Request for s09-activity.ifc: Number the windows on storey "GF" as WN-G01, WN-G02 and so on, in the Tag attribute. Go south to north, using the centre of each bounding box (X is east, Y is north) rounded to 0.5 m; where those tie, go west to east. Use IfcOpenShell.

First a look at what the model holds.

```python
import ifcopenshell
import ifcopenshell.util.element
import ifcopenshell.util.placement

model = ifcopenshell.open("s09-activity.ifc")
print(model.schema)
storey = next(s for s in model.by_type("IfcBuildingStorey") if s.Name == "GF")
windows = [e for e in ifcopenshell.util.element.get_decomposition(storey) if e.is_a("IfcWindow")]
for e in sorted(windows, key=lambda e: e.id()):
    origin = ifcopenshell.util.placement.get_local_placement(e.ObjectPlacement)[:3, 3]
    print(e.id(), e.Tag, e.Name, origin.round(2) + 0.0, sep=" | ")
```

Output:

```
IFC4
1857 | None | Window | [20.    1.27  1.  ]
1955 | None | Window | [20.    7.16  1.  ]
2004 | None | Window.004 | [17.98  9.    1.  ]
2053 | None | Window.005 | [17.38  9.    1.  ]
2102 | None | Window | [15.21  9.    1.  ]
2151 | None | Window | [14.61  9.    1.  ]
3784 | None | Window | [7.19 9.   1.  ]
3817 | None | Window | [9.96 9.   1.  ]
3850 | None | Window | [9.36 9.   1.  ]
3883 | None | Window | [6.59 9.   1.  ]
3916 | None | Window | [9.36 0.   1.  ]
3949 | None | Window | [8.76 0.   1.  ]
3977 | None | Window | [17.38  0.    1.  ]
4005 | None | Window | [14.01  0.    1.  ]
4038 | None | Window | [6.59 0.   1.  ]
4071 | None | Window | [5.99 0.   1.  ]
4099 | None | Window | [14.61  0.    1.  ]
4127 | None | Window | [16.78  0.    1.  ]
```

```python
import ifcopenshell
import ifcopenshell.geom
import ifcopenshell.util.element
import ifcopenshell.util.shape

model = ifcopenshell.open("s09-activity.ifc")
settings = ifcopenshell.geom.settings()
settings.set("use-world-coords", True)


def centre(element):
    shape = ifcopenshell.geom.create_shape(settings, element)
    return ifcopenshell.util.shape.get_bbox_centroid(shape.geometry)


storey = next(s for s in model.by_type("IfcBuildingStorey") if s.Name == "GF")
windows = [e for e in ifcopenshell.util.element.get_decomposition(storey) if e.is_a("IfcWindow")]

# Insertion points can sit at a corner or the storey origin, so sort by the geometry (in metres).
centres = {e: centre(e) for e in windows}
windows.sort(key=lambda e: (round(centres[e][1] / 0.5), centres[e][0]))

for i, e in enumerate(windows, start=1):
    number = f"WN-G{i:02d}"
    e.Tag = number
    print(e.id(), number)

model.write("s09-activity_updated.ifc")
```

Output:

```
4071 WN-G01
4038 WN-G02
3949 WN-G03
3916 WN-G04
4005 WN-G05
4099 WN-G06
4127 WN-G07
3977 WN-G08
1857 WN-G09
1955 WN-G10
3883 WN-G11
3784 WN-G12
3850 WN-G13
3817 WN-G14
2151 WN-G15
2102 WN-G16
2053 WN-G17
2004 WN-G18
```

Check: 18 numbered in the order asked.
